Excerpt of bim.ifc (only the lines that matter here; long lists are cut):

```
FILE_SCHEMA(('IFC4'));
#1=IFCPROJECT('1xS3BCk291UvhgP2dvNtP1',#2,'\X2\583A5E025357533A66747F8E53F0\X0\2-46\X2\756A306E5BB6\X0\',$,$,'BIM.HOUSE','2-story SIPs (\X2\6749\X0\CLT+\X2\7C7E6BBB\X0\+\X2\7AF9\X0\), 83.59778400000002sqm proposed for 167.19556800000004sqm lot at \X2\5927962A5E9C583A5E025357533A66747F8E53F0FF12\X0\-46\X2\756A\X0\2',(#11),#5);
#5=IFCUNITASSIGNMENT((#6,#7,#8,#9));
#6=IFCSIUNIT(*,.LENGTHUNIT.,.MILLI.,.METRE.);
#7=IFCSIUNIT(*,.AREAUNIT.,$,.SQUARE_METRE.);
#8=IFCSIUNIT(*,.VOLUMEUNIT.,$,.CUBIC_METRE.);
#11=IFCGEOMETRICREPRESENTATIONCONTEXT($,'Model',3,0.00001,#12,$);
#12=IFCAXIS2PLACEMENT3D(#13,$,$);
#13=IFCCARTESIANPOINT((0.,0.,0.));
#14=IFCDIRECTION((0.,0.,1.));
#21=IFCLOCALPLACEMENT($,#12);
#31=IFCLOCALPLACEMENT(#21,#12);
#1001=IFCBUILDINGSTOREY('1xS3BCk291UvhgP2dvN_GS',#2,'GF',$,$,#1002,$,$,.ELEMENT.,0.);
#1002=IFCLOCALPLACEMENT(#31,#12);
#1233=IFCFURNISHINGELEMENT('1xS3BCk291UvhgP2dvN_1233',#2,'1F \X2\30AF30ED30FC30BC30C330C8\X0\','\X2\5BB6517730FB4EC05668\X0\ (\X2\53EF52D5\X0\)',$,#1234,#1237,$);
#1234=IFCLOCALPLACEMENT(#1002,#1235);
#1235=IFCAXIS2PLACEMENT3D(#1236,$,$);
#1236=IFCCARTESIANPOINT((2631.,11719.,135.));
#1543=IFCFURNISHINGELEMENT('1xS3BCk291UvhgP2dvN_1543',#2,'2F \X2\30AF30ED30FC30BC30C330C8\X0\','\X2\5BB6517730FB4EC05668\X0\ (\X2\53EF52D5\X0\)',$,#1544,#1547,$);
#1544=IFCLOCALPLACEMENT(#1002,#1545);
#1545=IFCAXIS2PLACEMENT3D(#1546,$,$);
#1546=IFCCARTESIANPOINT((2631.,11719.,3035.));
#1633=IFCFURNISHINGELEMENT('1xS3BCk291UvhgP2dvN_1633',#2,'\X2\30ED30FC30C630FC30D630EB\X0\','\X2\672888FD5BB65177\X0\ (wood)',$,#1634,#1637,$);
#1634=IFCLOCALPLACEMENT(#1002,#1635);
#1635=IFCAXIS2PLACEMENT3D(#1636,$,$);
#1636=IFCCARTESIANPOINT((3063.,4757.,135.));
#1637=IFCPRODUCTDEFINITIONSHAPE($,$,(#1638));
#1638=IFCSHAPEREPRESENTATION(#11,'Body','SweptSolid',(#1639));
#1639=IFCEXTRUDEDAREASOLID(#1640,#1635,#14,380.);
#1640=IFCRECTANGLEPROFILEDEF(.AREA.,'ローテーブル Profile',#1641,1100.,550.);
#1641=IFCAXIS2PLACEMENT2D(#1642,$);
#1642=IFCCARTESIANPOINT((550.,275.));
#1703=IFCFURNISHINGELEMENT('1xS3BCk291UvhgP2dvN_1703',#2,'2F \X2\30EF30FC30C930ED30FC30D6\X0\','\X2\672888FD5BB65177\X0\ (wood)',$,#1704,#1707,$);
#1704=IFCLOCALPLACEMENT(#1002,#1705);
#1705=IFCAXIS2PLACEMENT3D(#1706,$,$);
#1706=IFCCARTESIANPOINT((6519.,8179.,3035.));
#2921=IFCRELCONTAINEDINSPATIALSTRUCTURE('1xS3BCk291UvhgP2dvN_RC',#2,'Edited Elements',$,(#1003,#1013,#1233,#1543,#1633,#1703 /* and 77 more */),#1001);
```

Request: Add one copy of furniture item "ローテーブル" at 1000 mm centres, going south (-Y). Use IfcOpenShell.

```python
import numpy as np
import ifcopenshell
import ifcopenshell.api.geometry
import ifcopenshell.api.root
import ifcopenshell.util.element
import ifcopenshell.util.placement

model = ifcopenshell.open("bim.ifc")


def reuse_history(source, copy):
    """copy_class also copies each property set's owner history, people and application; keep the originals."""
    for rel in copy.IsDefinedBy:
        if rel.is_a("IfcRelDefinesByProperties") and (history := rel.RelatingPropertyDefinition.OwnerHistory):
            rel.RelatingPropertyDefinition.OwnerHistory = source.OwnerHistory
            ifcopenshell.util.element.remove_deep2(model, history)


source = model.by_guid("1xS3BCk291UvhgP2dvN_1633")
base = ifcopenshell.util.placement.get_local_placement(source.ObjectPlacement)
step = np.array([0.0, -1.0, 0.0]) * 1000.0

for i in range(1, 2):
    copy = ifcopenshell.api.root.copy_class(model, product=source)
    copy.Representation = ifcopenshell.util.element.copy_deep(
        model, source.Representation, exclude=["IfcGeometricRepresentationContext", "IfcRepresentationMap"]
    )
    reuse_history(source, copy)
    matrix = base.copy()
    matrix[:3, 3] += i * step
    print("added at", matrix[:3, 3].round(3) + 0.0)
    ifcopenshell.api.geometry.edit_object_placement(model, product=copy, matrix=matrix, is_si=False)

model.write("bim_rev.ifc")
```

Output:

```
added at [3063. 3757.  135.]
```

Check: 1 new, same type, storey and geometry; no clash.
